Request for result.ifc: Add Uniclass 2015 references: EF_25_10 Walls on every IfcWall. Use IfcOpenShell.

First a look at what the model holds.

```python
import ifcopenshell

model = ifcopenshell.open("result.ifc")
print(model.schema)
print("classifications:", [c.Name for c in model.by_type("IfcClassification")])
for ifc_class in ("IfcDoor", "IfcRoof", "IfcStair", "IfcWall", "IfcWindow"):
    print(ifc_class, len(model.by_type(ifc_class)))
```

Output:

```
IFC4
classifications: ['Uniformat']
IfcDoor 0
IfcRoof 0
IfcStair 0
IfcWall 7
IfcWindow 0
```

```python
import ifcopenshell
import ifcopenshell.api.classification

model = ifcopenshell.open("result.ifc")

system = ifcopenshell.api.classification.add_classification(model, classification="Uniclass 2015")

codes = {
    "IfcWall": ("EF_25_10", "Walls"),
}
for ifc_class, (code, name) in codes.items():
    products = model.by_type(ifc_class)
    ifcopenshell.api.classification.add_reference(
        model, products=products, classification=system, identification=code, name=name
    )
    print(code, len(products))

model.write("result_edited.ifc")
```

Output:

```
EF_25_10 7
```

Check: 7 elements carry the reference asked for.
